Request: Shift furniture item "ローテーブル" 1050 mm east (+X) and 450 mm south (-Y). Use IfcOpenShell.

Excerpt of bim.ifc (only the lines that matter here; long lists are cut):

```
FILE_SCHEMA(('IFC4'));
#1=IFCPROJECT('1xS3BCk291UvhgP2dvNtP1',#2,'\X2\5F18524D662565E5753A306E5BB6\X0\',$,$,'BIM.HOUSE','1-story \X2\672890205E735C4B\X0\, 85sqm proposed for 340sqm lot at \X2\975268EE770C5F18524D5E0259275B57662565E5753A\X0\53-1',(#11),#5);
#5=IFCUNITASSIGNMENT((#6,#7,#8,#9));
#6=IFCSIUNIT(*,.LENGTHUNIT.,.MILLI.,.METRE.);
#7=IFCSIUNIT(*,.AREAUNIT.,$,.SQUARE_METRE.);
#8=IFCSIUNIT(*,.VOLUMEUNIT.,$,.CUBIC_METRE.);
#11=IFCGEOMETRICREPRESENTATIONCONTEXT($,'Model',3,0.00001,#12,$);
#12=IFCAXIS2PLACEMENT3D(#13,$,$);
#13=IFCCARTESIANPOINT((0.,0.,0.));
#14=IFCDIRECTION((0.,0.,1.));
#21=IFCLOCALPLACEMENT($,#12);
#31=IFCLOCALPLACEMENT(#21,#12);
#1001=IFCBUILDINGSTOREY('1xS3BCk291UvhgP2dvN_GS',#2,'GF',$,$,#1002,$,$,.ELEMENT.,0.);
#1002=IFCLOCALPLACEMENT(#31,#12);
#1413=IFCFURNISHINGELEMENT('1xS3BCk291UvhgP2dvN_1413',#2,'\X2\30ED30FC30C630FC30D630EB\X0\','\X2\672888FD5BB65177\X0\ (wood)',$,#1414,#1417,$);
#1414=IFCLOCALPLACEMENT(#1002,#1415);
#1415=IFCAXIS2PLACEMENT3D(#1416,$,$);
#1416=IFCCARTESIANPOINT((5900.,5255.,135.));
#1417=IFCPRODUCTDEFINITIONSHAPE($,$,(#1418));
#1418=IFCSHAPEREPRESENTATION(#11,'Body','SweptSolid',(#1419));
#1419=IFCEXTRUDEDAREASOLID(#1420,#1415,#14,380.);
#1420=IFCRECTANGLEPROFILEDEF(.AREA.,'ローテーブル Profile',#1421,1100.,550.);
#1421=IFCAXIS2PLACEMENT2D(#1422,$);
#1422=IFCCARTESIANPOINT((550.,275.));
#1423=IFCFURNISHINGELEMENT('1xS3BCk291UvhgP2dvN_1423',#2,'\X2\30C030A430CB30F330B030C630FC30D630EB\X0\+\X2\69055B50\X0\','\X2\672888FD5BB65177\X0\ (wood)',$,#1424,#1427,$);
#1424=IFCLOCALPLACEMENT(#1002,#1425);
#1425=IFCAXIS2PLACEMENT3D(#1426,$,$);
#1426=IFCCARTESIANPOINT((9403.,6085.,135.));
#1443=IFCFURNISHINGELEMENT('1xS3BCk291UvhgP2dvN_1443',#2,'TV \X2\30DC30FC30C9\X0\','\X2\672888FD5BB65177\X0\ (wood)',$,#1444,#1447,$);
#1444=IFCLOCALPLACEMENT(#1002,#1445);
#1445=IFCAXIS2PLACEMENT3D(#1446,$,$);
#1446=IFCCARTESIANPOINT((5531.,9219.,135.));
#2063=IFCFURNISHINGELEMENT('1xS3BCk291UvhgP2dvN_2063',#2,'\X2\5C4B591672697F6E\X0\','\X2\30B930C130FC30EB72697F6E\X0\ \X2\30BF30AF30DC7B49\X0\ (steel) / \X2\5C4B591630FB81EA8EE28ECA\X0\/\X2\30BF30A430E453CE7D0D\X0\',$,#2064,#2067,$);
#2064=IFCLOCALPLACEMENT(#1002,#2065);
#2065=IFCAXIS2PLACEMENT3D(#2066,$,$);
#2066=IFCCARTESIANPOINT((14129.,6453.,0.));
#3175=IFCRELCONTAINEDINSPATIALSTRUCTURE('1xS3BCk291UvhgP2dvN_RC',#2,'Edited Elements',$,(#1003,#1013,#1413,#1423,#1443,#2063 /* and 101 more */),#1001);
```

```python
import ifcopenshell
import ifcopenshell.api.geometry
import ifcopenshell.util.placement
import ifcopenshell.util.unit

model = ifcopenshell.open("bim.ifc")
unit_scale = ifcopenshell.util.unit.calculate_unit_scale(model)

item = model.by_guid("1xS3BCk291UvhgP2dvN_1413")
matrix = ifcopenshell.util.placement.get_local_placement(item.ObjectPlacement)
matrix[0, 3] += 1.05 / unit_scale
matrix[1, 3] -= 0.45 / unit_scale
ifcopenshell.api.geometry.edit_object_placement(model, product=item, matrix=matrix, is_si=False)

print(ifcopenshell.util.placement.get_local_placement(item.ObjectPlacement).round(3) + 0.0)

model.write("bim-out.ifc")
```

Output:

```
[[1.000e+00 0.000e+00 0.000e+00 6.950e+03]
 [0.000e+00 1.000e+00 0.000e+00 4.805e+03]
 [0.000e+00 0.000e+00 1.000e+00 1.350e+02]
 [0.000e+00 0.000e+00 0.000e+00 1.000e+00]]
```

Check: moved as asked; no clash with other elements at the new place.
